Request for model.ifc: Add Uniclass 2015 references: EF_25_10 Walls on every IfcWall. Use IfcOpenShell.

First a look at what the model holds.

```python
import ifcopenshell

model = ifcopenshell.open("model.ifc")
print(model.schema)
print("classifications:", [c.Name for c in model.by_type("IfcClassification")])
for ifc_class in ("IfcDoor", "IfcRoof", "IfcStair", "IfcWall", "IfcWindow"):
    print(ifc_class, len(model.by_type(ifc_class)))
```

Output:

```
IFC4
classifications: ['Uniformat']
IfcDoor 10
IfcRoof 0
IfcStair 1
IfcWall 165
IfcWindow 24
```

```python
import ifcopenshell
import ifcopenshell.api.classification

model = ifcopenshell.open("model.ifc")

system = ifcopenshell.api.classification.add_classification(model, classification="Uniclass 2015")

codes = {
    "IfcWall": ("EF_25_10", "Walls"),
}
for ifc_class, (code, name) in codes.items():
    products = model.by_type(ifc_class)
    ifcopenshell.api.classification.add_reference(
        model, products=products, classification=system, identification=code, name=name
    )
    print(code, len(products))

model.write("model_rev.ifc")
```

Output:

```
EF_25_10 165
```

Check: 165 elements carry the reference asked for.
